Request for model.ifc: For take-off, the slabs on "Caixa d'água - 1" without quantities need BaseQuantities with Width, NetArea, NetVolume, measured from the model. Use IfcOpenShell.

First a look at what the model holds.

```python
import ifcopenshell
import ifcopenshell.util.element
import ifcopenshell.util.unit

model = ifcopenshell.open("model.ifc")
print(model.schema)
for unit_type in ("LENGTHUNIT", "AREAUNIT", "VOLUMEUNIT"):
    print(unit_type, ifcopenshell.util.unit.calculate_unit_scale(model, unit_type))
storey = next(s for s in model.by_type("IfcBuildingStorey") if s.Name == "Caixa d'água - 1")
slabs = [e for e in ifcopenshell.util.element.get_decomposition(storey) if e.is_a("IfcSlab")]
for e in sorted(slabs, key=lambda e: e.id()):
    print(e.id(), e.is_a(), e.Name, list(ifcopenshell.util.element.get_psets(e, qtos_only=True)), sep=" | ")
```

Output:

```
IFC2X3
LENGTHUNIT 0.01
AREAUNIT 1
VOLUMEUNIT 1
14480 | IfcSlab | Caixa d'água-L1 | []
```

```python
import ifcopenshell
import ifcopenshell.api.pset
import ifcopenshell.geom
import ifcopenshell.util.element
import ifcopenshell.util.shape
import ifcopenshell.util.unit

model = ifcopenshell.open("model.ifc")
unit_scale = ifcopenshell.util.unit.calculate_unit_scale(model)
area_scale = ifcopenshell.util.unit.calculate_unit_scale(model, "AREAUNIT")
volume_scale = ifcopenshell.util.unit.calculate_unit_scale(model, "VOLUMEUNIT")
settings = ifcopenshell.geom.settings()

storey = next(s for s in model.by_type("IfcBuildingStorey") if s.Name == "Caixa d'água - 1")
slabs = [e for e in ifcopenshell.util.element.get_decomposition(storey) if e.is_a("IfcSlab")]

for e in sorted(slabs, key=lambda e: e.id()):
    if ifcopenshell.util.element.get_psets(e, qtos_only=True, should_inherit=False):
        continue
    # Geometry comes back in metres, in the element's own axes.
    shape = ifcopenshell.geom.create_shape(settings, e)
    values = {
        "Width": ifcopenshell.util.shape.get_z(shape.geometry) / unit_scale,
        "NetArea": ifcopenshell.util.shape.get_footprint_area(shape.geometry) / area_scale,
        "NetVolume": ifcopenshell.util.shape.get_volume(shape.geometry) / volume_scale,
    }
    qto = ifcopenshell.api.pset.add_qto(model, product=e, name="BaseQuantities")
    ifcopenshell.api.pset.edit_qto(model, qto=qto, properties=values)
    print(e.id(), {k: round(v, 3) for k, v in values.items()})

model.write("model-out.ifc")
```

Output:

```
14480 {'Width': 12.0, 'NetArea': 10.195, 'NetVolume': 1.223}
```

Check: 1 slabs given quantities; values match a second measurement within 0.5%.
